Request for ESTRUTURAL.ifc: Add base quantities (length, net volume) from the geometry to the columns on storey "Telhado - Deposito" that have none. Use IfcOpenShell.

First a look at what the model holds.

```python
import ifcopenshell
import ifcopenshell.util.element
import ifcopenshell.util.unit

model = ifcopenshell.open("ESTRUTURAL.ifc")
print(model.schema)
for unit_type in ("LENGTHUNIT", "AREAUNIT", "VOLUMEUNIT"):
    print(unit_type, ifcopenshell.util.unit.calculate_unit_scale(model, unit_type))
storey = next(s for s in model.by_type("IfcBuildingStorey") if s.Name == "Telhado - Deposito")
columns = [e for e in ifcopenshell.util.element.get_decomposition(storey) if e.is_a("IfcColumn")]
for e in sorted(columns, key=lambda e: e.id()):
    print(e.id(), e.is_a(), e.Name, list(ifcopenshell.util.element.get_psets(e, qtos_only=True)), sep=" | ")
```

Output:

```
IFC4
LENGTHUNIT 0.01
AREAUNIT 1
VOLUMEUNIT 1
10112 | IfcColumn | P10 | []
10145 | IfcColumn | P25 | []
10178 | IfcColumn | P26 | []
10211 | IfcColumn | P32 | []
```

```python
import ifcopenshell
import ifcopenshell.api.pset
import ifcopenshell.geom
import ifcopenshell.util.element
import ifcopenshell.util.shape
import ifcopenshell.util.unit

model = ifcopenshell.open("ESTRUTURAL.ifc")
unit_scale = ifcopenshell.util.unit.calculate_unit_scale(model)
volume_scale = ifcopenshell.util.unit.calculate_unit_scale(model, "VOLUMEUNIT")
settings = ifcopenshell.geom.settings()

storey = next(s for s in model.by_type("IfcBuildingStorey") if s.Name == "Telhado - Deposito")
columns = [e for e in ifcopenshell.util.element.get_decomposition(storey) if e.is_a("IfcColumn")]

for e in sorted(columns, key=lambda e: e.id()):
    if ifcopenshell.util.element.get_psets(e, qtos_only=True, should_inherit=False):
        continue
    # Geometry comes back in metres, in the element's own axes.
    shape = ifcopenshell.geom.create_shape(settings, e)
    values = {
        "Length": ifcopenshell.util.shape.get_z(shape.geometry) / unit_scale,
        "NetVolume": ifcopenshell.util.shape.get_volume(shape.geometry) / volume_scale,
    }
    qto = ifcopenshell.api.pset.add_qto(model, product=e, name="Qto_ColumnBaseQuantities")
    ifcopenshell.api.pset.edit_qto(model, qto=qto, properties=values)
    print(e.id(), {k: round(v, 3) for k, v in values.items()})

model.write("ESTRUTURAL_v2.ifc")
```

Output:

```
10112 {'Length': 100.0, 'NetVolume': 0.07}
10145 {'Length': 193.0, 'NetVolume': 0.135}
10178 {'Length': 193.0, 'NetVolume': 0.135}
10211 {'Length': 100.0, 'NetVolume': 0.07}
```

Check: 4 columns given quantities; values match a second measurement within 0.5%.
